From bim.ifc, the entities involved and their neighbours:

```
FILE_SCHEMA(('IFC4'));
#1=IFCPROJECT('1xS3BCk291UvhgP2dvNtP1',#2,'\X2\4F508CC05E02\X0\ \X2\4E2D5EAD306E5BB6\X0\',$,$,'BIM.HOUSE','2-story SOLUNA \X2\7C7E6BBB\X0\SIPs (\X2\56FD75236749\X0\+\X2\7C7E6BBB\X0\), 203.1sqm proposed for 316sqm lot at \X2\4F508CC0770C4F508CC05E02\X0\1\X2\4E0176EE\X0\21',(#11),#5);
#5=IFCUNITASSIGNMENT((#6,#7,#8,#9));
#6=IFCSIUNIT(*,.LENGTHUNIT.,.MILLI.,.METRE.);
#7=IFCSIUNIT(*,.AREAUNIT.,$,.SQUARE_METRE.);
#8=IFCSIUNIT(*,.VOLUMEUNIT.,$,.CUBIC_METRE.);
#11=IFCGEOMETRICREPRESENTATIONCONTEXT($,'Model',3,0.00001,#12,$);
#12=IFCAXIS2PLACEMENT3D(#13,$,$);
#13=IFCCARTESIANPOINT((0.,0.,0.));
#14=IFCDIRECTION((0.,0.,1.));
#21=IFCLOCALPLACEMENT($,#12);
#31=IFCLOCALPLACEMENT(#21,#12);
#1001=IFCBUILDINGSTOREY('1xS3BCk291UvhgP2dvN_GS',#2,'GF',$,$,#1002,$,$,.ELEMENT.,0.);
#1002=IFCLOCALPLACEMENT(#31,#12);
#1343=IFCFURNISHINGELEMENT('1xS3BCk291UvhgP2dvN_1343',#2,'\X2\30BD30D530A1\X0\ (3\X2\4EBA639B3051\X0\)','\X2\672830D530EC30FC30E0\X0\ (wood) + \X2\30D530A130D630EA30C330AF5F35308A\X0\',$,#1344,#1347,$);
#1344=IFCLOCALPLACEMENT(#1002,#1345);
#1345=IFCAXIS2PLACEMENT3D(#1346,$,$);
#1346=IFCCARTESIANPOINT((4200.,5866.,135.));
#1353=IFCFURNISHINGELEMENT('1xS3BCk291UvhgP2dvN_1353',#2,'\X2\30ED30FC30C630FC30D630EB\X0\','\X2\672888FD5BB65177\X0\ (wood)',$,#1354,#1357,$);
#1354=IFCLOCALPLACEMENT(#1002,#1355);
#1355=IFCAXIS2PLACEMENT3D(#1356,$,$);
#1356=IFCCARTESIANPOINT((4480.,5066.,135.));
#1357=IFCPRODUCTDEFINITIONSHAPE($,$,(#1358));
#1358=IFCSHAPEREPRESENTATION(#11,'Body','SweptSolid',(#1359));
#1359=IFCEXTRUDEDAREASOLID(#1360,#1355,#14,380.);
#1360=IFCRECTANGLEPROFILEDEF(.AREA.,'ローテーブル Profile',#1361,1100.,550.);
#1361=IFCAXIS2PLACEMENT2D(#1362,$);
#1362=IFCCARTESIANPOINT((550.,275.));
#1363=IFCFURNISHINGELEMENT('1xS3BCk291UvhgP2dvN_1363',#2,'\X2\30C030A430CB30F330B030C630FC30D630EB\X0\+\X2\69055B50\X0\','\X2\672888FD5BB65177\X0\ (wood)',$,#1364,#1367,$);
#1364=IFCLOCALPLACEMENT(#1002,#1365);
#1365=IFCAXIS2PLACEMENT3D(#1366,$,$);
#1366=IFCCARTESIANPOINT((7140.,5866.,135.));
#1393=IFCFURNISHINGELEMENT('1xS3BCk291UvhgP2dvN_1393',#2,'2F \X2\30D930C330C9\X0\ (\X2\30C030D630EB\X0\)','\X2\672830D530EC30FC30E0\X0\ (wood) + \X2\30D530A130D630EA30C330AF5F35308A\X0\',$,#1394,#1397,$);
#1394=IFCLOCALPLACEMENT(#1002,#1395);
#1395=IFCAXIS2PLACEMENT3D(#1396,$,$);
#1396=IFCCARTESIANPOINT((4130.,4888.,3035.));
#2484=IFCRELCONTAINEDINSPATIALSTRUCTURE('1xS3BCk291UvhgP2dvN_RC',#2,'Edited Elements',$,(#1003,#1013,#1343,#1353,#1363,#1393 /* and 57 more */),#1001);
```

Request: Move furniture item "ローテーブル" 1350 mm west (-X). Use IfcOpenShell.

```python
import ifcopenshell
import ifcopenshell.api.geometry
import ifcopenshell.util.placement
import ifcopenshell.util.unit

model = ifcopenshell.open("bim.ifc")
unit_scale = ifcopenshell.util.unit.calculate_unit_scale(model)

item = model.by_guid("1xS3BCk291UvhgP2dvN_1353")
matrix = ifcopenshell.util.placement.get_local_placement(item.ObjectPlacement)
matrix[0, 3] -= 1.35 / unit_scale
ifcopenshell.api.geometry.edit_object_placement(model, product=item, matrix=matrix, is_si=False)

print(ifcopenshell.util.placement.get_local_placement(item.ObjectPlacement).round(3) + 0.0)

model.write("bim_v2.ifc")
```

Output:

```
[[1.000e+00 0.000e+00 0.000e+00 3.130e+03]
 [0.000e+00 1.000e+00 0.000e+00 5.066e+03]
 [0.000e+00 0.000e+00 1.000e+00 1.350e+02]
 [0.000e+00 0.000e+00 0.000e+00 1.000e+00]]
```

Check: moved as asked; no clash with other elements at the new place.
